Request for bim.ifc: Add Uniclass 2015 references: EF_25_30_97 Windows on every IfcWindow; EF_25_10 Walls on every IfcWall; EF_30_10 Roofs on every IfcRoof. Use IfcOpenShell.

First a look at what the model holds.

```python
import ifcopenshell

model = ifcopenshell.open("bim.ifc")
print(model.schema)
print("classifications:", [c.Name for c in model.by_type("IfcClassification")])
for ifc_class in ("IfcDoor", "IfcRoof", "IfcStair", "IfcWall", "IfcWindow"):
    print(ifc_class, len(model.by_type(ifc_class)))
```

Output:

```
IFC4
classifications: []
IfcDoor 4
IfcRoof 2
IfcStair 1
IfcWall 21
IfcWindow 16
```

```python
import ifcopenshell
import ifcopenshell.api.classification

model = ifcopenshell.open("bim.ifc")

system = ifcopenshell.api.classification.add_classification(model, classification="Uniclass 2015")

codes = {
    "IfcWindow": ("EF_25_30_97", "Windows"),
    "IfcWall": ("EF_25_10", "Walls"),
    "IfcRoof": ("EF_30_10", "Roofs"),
}
for ifc_class, (code, name) in codes.items():
    products = model.by_type(ifc_class)
    ifcopenshell.api.classification.add_reference(
        model, products=products, classification=system, identification=code, name=name
    )
    print(code, len(products))

model.write("bim_v2.ifc")
```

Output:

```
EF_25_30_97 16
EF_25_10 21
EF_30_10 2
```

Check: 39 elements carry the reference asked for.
